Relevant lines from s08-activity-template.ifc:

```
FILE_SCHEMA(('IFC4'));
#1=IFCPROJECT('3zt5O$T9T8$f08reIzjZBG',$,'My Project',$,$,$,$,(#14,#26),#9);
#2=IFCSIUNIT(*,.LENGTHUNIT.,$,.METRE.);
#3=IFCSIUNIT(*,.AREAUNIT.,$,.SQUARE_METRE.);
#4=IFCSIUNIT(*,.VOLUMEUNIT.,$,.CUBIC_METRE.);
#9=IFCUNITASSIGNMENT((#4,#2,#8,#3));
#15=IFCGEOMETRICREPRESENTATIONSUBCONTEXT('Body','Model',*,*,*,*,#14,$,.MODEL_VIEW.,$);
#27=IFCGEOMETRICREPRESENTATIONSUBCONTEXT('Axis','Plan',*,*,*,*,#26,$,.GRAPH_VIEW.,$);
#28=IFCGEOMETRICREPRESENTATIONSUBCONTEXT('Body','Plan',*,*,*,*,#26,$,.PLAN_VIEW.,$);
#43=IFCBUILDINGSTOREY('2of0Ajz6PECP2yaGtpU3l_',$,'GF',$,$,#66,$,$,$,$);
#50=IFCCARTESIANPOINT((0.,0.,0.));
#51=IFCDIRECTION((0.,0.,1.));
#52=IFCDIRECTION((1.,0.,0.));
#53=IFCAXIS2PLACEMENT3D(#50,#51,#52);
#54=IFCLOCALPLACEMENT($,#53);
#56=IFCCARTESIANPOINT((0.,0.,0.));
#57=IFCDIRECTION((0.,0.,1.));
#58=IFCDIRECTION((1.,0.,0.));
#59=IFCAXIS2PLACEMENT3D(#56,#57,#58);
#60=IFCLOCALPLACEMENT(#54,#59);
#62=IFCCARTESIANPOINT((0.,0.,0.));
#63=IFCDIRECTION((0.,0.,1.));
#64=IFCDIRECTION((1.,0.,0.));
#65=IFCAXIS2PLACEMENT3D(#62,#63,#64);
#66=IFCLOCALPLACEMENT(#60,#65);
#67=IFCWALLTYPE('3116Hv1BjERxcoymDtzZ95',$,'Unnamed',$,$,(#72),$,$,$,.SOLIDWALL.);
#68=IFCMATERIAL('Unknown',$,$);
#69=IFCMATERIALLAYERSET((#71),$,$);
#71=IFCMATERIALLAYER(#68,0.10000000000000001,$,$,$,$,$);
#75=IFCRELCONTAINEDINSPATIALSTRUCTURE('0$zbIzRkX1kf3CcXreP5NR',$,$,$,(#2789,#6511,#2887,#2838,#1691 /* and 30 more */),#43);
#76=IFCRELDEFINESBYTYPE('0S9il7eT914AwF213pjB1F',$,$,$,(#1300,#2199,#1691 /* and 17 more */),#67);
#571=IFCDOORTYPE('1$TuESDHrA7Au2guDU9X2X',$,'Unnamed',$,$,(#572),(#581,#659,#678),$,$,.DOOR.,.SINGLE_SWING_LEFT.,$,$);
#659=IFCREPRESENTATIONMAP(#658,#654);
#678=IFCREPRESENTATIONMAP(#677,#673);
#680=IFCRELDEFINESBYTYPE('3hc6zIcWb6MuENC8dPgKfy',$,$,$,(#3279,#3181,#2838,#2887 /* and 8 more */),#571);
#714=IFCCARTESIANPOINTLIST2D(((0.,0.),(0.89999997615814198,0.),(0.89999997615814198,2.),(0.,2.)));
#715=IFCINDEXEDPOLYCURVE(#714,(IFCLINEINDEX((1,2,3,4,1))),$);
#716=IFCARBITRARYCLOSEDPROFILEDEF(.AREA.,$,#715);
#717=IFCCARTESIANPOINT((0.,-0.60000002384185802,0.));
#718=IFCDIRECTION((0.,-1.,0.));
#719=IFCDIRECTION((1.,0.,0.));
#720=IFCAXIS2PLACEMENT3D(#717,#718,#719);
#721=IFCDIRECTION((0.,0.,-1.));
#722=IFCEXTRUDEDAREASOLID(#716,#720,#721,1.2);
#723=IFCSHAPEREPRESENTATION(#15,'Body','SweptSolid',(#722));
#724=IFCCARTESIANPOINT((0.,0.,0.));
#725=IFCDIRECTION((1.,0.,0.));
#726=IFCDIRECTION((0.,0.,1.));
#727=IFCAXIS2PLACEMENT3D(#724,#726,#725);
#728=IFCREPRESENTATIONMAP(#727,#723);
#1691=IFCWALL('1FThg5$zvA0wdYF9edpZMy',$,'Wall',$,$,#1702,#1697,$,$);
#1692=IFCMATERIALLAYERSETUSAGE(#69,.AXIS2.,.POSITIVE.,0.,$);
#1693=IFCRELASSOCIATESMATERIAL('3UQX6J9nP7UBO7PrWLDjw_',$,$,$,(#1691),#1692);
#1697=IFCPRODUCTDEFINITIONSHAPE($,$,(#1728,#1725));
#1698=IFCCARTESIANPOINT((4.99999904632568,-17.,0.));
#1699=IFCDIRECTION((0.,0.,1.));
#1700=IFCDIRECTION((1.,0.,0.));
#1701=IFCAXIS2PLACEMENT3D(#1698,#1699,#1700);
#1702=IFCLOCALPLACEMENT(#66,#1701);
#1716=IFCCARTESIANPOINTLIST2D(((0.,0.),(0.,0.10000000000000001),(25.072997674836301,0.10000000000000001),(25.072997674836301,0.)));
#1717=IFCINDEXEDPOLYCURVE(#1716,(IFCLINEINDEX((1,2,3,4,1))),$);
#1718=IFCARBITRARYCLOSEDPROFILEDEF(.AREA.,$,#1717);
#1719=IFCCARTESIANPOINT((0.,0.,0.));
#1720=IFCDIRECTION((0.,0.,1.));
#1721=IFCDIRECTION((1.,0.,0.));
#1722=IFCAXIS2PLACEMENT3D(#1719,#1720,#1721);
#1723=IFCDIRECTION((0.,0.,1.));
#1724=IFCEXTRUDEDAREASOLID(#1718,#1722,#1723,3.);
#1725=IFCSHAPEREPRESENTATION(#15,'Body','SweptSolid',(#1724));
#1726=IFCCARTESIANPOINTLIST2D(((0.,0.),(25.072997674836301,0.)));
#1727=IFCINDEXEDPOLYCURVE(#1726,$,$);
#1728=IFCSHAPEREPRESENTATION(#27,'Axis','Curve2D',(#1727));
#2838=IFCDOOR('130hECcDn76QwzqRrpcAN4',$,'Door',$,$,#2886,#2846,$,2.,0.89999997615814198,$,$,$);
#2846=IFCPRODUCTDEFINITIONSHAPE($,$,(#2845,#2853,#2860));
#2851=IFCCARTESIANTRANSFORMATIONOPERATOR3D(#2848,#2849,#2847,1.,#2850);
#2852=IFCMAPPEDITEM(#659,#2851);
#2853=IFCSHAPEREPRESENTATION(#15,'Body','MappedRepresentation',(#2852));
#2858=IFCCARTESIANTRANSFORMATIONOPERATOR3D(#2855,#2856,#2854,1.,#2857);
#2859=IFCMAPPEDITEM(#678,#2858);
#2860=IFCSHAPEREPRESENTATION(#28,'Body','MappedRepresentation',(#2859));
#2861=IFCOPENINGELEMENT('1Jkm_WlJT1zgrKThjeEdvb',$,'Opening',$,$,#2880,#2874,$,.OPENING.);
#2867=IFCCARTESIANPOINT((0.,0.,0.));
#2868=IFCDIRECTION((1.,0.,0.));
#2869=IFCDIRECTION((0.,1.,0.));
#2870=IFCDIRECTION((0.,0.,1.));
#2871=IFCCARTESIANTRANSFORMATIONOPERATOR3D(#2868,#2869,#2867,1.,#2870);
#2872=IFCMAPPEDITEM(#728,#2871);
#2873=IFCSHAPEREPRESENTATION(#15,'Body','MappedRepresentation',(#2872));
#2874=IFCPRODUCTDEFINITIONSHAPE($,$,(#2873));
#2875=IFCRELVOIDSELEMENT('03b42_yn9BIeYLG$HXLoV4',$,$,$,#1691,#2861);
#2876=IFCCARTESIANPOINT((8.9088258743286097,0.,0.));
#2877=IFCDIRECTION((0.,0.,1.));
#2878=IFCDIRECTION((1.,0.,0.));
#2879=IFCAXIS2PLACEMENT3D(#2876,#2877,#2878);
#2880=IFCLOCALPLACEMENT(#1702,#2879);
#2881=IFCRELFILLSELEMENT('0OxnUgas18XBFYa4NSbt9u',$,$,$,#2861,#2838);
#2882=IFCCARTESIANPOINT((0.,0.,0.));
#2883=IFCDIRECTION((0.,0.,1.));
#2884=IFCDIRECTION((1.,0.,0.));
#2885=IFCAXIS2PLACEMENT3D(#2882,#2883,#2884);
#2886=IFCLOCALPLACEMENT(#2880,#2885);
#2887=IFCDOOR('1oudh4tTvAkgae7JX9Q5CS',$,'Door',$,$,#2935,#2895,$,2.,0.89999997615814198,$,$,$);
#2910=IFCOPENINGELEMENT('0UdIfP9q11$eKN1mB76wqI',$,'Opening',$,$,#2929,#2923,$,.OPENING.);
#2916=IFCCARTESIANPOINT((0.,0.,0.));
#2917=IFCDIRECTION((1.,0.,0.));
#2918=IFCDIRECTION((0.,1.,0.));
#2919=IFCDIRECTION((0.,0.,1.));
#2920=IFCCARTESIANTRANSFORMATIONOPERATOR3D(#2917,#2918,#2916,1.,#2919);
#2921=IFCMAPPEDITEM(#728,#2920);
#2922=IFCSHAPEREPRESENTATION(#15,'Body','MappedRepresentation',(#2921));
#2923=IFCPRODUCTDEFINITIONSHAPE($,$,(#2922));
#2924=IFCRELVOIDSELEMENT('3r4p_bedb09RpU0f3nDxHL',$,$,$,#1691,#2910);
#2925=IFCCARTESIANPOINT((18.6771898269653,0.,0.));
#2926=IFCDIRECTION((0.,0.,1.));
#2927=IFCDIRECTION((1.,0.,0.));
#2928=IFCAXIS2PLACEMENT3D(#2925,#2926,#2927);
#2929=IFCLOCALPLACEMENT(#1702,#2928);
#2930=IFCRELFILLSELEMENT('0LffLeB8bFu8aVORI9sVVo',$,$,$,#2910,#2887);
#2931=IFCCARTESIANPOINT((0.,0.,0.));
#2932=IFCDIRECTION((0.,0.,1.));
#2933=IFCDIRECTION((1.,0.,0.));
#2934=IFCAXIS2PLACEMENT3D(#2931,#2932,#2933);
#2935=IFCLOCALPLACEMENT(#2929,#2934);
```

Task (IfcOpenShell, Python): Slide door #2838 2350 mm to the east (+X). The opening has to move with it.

```python
import ifcopenshell
import ifcopenshell.api.geometry
import ifcopenshell.util.placement

model = ifcopenshell.open("s08-activity-template.ifc")

door = model.by_guid("130hECcDn76QwzqRrpcAN4")
opening = door.FillsVoids[0].RelatingOpeningElement
wall = opening.VoidsElements[0].RelatingBuildingElement

wall_matrix = ifcopenshell.util.placement.get_local_placement(wall.ObjectPlacement)
shift = wall_matrix[:3, 0] * 2.35
before = ifcopenshell.util.placement.get_local_placement(door.ObjectPlacement)[:3, 3].copy()

# The door is placed relative to its opening, so it follows when the opening moves.
matrix = ifcopenshell.util.placement.get_local_placement(opening.ObjectPlacement)
matrix[:3, 3] += shift
ifcopenshell.api.geometry.edit_object_placement(
    model, product=opening, matrix=matrix, is_si=False, should_transform_children=True
)

after = ifcopenshell.util.placement.get_local_placement(door.ObjectPlacement)[:3, 3]
print("door moved by", (after - before).round(3) + 0.0)

model.write("s08-activity-template_edited.ifc")
```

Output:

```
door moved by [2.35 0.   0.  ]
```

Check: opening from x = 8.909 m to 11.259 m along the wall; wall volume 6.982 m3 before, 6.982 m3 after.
